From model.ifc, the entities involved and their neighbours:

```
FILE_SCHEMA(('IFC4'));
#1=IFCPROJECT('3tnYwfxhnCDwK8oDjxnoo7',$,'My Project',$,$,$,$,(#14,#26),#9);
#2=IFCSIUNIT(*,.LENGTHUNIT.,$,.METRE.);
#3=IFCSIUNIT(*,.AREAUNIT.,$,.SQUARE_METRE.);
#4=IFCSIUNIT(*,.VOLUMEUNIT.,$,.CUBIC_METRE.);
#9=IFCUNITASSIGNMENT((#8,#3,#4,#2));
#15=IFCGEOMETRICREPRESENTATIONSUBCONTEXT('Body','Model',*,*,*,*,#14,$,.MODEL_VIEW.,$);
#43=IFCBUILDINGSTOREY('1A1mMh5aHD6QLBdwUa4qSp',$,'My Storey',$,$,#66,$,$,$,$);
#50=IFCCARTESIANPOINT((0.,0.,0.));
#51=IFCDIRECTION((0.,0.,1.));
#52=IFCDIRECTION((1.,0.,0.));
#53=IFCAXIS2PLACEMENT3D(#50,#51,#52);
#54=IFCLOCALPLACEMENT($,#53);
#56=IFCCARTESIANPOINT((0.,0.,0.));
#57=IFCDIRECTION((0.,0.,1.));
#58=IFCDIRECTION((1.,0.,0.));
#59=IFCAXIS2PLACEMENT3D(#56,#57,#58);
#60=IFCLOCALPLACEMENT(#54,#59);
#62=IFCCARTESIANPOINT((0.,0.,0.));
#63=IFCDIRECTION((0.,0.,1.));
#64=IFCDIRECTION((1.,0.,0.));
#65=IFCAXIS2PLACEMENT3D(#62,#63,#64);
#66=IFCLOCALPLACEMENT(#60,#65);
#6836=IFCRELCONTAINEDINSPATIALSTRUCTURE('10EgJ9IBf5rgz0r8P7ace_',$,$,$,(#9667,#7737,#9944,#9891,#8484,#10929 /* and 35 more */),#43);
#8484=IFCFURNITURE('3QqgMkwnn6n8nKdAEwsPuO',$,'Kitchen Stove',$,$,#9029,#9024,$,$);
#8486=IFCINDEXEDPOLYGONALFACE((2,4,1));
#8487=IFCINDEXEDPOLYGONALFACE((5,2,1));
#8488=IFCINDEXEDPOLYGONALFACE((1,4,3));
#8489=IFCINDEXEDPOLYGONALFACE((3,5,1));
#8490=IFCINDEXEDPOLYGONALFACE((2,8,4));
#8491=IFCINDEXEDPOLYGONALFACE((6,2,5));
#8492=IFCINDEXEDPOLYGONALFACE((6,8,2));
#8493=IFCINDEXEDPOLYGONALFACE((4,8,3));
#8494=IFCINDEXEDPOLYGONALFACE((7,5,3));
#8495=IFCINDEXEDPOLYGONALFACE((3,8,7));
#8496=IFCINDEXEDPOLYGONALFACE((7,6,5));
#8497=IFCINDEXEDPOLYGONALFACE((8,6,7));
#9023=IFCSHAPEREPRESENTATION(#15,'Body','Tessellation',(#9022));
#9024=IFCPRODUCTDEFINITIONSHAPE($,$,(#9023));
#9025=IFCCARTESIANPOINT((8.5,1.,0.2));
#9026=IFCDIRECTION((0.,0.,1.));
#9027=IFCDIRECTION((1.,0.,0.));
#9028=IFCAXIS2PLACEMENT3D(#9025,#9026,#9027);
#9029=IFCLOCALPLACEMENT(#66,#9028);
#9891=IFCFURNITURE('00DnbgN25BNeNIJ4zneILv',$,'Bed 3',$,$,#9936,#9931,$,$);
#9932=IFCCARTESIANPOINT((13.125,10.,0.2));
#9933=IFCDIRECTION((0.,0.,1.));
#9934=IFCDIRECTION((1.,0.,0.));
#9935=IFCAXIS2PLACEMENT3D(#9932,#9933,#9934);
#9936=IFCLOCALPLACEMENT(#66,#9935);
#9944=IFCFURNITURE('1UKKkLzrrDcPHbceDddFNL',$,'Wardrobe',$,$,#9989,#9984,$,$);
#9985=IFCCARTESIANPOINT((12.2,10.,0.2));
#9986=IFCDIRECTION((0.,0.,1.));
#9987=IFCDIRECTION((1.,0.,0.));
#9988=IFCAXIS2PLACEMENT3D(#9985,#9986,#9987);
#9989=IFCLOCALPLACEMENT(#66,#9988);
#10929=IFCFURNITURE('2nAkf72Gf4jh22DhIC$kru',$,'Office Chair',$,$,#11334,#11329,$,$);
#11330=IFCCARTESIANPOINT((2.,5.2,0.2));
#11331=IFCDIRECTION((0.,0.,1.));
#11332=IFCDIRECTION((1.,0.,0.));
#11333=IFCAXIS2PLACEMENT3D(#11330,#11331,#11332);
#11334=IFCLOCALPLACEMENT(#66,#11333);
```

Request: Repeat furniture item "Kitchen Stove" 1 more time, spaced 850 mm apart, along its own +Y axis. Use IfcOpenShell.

```python
import ifcopenshell
import ifcopenshell.api.geometry
import ifcopenshell.api.root
import ifcopenshell.util.element
import ifcopenshell.util.placement
import ifcopenshell.util.unit

model = ifcopenshell.open("model.ifc")
unit_scale = ifcopenshell.util.unit.calculate_unit_scale(model)

source = model.by_guid("3QqgMkwnn6n8nKdAEwsPuO")
base = ifcopenshell.util.placement.get_local_placement(source.ObjectPlacement)
step = base[:3, 1] * 0.85 / unit_scale

for i in range(1, 2):
    copy = ifcopenshell.api.root.copy_class(model, product=source)
    copy.Representation = ifcopenshell.util.element.copy_deep(
        model, source.Representation, exclude=["IfcGeometricRepresentationContext", "IfcRepresentationMap"]
    )
    matrix = base.copy()
    matrix[:3, 3] += i * step
    print("added at", matrix[:3, 3].round(3) + 0.0)
    ifcopenshell.api.geometry.edit_object_placement(model, product=copy, matrix=matrix, is_si=False)

model.write("model_edited.ifc")
```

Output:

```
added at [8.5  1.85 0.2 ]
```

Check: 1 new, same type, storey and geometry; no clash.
